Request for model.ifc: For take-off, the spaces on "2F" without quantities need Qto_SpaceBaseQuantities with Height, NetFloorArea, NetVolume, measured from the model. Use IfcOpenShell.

First a look at what the model holds.

```python
import ifcopenshell
import ifcopenshell.util.element
import ifcopenshell.util.unit

model = ifcopenshell.open("model.ifc")
print(model.schema)
for unit_type in ("LENGTHUNIT", "AREAUNIT", "VOLUMEUNIT"):
    print(unit_type, ifcopenshell.util.unit.calculate_unit_scale(model, unit_type))
storey = next(s for s in model.by_type("IfcBuildingStorey") if s.Name == "2F")
spaces = [e for e in ifcopenshell.util.element.get_decomposition(storey) if e.is_a("IfcSpace")]
for e in sorted(spaces, key=lambda e: e.id()):
    print(e.id(), e.is_a(), e.Name, list(ifcopenshell.util.element.get_psets(e, qtos_only=True)), sep=" | ")
```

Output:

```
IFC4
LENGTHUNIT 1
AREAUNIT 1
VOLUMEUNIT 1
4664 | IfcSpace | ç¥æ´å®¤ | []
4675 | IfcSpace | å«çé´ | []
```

```python
import ifcopenshell
import ifcopenshell.api.pset
import ifcopenshell.geom
import ifcopenshell.util.element
import ifcopenshell.util.shape
import ifcopenshell.util.unit

model = ifcopenshell.open("model.ifc")
unit_scale = ifcopenshell.util.unit.calculate_unit_scale(model)
area_scale = ifcopenshell.util.unit.calculate_unit_scale(model, "AREAUNIT")
volume_scale = ifcopenshell.util.unit.calculate_unit_scale(model, "VOLUMEUNIT")
settings = ifcopenshell.geom.settings()

storey = next(s for s in model.by_type("IfcBuildingStorey") if s.Name == "2F")
spaces = [e for e in ifcopenshell.util.element.get_decomposition(storey) if e.is_a("IfcSpace")]

for e in sorted(spaces, key=lambda e: e.id()):
    if ifcopenshell.util.element.get_psets(e, qtos_only=True, should_inherit=False):
        continue
    # Geometry comes back in metres, in the element's own axes.
    shape = ifcopenshell.geom.create_shape(settings, e)
    values = {
        "Height": ifcopenshell.util.shape.get_z(shape.geometry) / unit_scale,
        "NetFloorArea": ifcopenshell.util.shape.get_footprint_area(shape.geometry) / area_scale,
        "NetVolume": ifcopenshell.util.shape.get_volume(shape.geometry) / volume_scale,
    }
    qto = ifcopenshell.api.pset.add_qto(model, product=e, name="Qto_SpaceBaseQuantities")
    ifcopenshell.api.pset.edit_qto(model, qto=qto, properties=values)
    print(e.id(), {k: round(v, 3) for k, v in values.items()})

model.write("model-out.ifc")
```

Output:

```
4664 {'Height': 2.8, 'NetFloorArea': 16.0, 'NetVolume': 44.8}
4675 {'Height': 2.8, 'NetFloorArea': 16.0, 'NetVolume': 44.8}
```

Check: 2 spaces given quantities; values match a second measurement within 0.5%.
